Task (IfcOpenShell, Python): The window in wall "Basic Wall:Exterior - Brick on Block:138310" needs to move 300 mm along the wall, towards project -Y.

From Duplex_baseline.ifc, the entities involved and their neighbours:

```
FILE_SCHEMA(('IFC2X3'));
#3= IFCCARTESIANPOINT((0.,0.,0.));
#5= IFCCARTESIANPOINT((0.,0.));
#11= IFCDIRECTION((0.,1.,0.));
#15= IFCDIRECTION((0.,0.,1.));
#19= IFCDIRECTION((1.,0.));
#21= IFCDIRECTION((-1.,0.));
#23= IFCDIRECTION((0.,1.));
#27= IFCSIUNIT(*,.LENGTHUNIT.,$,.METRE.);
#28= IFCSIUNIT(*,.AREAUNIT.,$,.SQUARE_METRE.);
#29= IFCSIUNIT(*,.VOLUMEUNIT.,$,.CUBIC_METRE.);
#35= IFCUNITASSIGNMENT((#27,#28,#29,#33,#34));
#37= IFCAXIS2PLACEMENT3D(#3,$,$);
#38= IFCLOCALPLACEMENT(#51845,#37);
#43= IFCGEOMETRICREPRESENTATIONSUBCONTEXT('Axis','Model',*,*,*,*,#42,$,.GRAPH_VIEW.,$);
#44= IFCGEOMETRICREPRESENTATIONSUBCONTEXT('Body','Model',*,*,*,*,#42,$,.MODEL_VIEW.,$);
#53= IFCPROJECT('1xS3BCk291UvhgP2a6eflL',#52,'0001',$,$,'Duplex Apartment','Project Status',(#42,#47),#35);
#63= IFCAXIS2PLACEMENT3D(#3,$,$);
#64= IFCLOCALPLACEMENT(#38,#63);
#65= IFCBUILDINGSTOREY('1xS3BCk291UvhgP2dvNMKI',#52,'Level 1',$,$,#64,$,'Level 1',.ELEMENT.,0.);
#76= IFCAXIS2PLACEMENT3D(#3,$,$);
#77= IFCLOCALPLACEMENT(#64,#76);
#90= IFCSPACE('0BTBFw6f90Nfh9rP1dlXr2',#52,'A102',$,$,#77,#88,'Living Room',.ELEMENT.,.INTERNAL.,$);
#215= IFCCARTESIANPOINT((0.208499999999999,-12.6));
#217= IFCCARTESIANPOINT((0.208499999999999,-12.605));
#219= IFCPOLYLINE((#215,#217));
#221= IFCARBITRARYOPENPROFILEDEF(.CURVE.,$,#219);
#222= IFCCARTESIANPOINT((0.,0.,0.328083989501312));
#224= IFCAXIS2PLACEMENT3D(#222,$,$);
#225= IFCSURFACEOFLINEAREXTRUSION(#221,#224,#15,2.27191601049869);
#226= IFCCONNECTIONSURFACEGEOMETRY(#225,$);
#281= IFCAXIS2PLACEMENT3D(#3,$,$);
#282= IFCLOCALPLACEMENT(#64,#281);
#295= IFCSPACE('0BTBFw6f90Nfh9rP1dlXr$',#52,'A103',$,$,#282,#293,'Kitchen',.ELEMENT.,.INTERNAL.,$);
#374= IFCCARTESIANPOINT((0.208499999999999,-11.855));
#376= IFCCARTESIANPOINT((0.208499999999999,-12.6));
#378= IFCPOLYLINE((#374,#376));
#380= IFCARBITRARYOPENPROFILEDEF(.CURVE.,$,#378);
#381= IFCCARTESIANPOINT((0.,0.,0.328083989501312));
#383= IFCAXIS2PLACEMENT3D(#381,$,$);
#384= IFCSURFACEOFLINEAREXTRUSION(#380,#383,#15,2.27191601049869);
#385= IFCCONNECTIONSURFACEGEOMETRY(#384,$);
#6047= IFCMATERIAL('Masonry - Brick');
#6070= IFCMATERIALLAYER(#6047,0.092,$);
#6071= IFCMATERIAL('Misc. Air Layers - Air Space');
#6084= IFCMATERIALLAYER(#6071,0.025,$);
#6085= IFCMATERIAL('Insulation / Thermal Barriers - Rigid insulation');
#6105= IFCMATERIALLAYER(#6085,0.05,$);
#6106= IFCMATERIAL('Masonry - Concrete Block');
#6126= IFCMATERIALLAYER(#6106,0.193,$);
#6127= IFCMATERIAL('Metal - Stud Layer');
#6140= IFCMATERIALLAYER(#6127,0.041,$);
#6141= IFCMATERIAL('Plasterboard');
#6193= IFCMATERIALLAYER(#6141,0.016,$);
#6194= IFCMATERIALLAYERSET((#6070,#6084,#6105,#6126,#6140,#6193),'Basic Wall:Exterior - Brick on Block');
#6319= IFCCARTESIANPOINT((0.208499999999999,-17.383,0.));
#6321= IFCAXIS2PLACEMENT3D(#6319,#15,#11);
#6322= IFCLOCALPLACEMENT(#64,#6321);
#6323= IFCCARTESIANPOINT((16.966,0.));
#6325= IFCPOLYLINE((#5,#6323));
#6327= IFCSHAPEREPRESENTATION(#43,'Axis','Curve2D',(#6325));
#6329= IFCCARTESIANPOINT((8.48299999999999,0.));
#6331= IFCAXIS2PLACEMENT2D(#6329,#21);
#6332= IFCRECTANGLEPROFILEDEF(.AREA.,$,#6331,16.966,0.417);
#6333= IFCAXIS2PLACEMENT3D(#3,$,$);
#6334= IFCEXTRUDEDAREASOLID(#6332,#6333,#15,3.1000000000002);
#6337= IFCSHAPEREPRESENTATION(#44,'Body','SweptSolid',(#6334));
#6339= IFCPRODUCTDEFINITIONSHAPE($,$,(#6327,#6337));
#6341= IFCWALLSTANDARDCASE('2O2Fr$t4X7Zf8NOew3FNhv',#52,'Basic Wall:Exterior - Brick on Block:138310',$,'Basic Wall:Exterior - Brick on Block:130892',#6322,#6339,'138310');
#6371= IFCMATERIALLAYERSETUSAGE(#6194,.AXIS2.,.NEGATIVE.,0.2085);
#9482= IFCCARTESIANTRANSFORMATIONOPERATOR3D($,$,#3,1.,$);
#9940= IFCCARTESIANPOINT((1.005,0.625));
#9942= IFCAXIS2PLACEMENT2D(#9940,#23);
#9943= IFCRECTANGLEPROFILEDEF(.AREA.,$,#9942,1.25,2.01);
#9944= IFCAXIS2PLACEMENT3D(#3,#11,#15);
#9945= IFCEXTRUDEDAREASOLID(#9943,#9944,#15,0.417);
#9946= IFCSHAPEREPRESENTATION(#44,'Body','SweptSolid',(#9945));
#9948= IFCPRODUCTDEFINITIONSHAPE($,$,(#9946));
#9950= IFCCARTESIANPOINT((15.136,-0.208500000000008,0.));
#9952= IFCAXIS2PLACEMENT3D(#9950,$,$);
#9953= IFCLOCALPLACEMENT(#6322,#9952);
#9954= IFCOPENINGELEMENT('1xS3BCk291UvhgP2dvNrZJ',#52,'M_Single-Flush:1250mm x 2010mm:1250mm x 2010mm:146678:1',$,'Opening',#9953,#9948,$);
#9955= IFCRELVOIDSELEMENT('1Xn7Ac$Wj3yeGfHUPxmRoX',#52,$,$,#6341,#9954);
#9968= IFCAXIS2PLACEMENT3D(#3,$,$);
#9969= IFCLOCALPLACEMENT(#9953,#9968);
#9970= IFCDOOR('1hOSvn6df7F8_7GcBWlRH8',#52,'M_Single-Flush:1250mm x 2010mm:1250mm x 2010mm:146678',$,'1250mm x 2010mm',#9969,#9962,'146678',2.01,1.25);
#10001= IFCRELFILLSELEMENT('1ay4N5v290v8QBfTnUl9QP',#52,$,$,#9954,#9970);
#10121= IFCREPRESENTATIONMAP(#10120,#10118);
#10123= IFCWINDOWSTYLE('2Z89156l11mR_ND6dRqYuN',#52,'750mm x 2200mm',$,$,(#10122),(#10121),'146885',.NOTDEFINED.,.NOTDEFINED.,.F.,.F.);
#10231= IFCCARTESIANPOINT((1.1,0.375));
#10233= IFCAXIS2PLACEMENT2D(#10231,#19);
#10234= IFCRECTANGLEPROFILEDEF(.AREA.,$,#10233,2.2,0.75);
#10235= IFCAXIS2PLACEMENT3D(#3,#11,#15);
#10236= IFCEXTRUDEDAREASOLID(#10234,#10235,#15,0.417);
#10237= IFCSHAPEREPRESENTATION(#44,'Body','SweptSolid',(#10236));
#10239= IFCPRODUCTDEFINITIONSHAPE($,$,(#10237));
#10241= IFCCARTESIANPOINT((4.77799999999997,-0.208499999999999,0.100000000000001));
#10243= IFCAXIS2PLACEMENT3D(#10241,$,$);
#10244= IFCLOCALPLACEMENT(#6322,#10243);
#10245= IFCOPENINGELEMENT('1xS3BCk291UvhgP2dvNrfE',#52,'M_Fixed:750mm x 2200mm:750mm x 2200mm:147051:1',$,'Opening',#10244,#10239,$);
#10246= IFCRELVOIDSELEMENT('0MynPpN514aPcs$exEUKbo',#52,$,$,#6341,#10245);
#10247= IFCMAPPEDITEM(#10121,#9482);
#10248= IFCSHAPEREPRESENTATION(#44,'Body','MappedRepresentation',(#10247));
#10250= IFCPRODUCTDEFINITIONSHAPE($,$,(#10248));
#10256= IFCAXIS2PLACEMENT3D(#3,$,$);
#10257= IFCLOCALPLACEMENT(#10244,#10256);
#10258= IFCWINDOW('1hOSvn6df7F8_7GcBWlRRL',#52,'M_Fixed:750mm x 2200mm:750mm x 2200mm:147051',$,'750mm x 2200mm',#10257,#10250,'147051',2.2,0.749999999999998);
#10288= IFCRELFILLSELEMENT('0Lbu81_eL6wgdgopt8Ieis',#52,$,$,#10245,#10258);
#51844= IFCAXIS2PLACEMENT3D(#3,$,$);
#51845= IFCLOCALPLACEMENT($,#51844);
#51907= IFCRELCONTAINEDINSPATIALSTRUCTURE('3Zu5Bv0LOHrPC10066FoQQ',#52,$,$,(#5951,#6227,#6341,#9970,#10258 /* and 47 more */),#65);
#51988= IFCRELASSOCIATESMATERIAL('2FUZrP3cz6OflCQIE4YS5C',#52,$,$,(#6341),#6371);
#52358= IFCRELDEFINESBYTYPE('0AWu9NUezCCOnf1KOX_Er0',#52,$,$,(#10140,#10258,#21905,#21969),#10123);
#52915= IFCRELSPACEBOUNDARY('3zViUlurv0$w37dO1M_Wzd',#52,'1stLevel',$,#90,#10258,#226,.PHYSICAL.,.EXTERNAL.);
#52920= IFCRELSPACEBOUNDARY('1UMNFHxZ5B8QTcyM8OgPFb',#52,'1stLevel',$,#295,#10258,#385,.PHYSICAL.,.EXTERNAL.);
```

```python
import numpy as np
import ifcopenshell
import ifcopenshell.api.geometry
import ifcopenshell.util.placement

model = ifcopenshell.open("Duplex_baseline.ifc")

window = model.by_guid("1hOSvn6df7F8_7GcBWlRRL")
opening = window.FillsVoids[0].RelatingOpeningElement
wall = opening.VoidsElements[0].RelatingBuildingElement

wall_matrix = ifcopenshell.util.placement.get_local_placement(wall.ObjectPlacement)
shift = wall_matrix[:3, 0] * -0.3
before = ifcopenshell.util.placement.get_local_placement(window.ObjectPlacement)[:3, 3].copy()

# The window is placed relative to its opening, so it follows when the opening moves.
matrix = ifcopenshell.util.placement.get_local_placement(opening.ObjectPlacement)
matrix[:3, 3] += shift
ifcopenshell.api.geometry.edit_object_placement(
    model, product=opening, matrix=matrix, is_si=False, should_transform_children=True
)

# Space boundary surfaces are stored in each space's coordinates; move them too.
for rel in window.ProvidesBoundaries:
    if not rel.ConnectionGeometry:
        continue
    surface = rel.ConnectionGeometry.SurfaceOnRelatingElement
    space_matrix = ifcopenshell.util.placement.get_local_placement(rel.RelatingSpace.ObjectPlacement)
    point = np.array(surface.Position.Location.Coordinates) + space_matrix[:3, :3].T @ shift
    surface.Position = model.createIfcAxis2Placement3D(
        model.createIfcCartesianPoint(point.tolist()), surface.Position.Axis, surface.Position.RefDirection
    )

after = ifcopenshell.util.placement.get_local_placement(window.ObjectPlacement)[:3, 3]
print("window moved by", (after - before).round(3) + 0.0)

model.write("Duplex_baseline-out.ifc")
```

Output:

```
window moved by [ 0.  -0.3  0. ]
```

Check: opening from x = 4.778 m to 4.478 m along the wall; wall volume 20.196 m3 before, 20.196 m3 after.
